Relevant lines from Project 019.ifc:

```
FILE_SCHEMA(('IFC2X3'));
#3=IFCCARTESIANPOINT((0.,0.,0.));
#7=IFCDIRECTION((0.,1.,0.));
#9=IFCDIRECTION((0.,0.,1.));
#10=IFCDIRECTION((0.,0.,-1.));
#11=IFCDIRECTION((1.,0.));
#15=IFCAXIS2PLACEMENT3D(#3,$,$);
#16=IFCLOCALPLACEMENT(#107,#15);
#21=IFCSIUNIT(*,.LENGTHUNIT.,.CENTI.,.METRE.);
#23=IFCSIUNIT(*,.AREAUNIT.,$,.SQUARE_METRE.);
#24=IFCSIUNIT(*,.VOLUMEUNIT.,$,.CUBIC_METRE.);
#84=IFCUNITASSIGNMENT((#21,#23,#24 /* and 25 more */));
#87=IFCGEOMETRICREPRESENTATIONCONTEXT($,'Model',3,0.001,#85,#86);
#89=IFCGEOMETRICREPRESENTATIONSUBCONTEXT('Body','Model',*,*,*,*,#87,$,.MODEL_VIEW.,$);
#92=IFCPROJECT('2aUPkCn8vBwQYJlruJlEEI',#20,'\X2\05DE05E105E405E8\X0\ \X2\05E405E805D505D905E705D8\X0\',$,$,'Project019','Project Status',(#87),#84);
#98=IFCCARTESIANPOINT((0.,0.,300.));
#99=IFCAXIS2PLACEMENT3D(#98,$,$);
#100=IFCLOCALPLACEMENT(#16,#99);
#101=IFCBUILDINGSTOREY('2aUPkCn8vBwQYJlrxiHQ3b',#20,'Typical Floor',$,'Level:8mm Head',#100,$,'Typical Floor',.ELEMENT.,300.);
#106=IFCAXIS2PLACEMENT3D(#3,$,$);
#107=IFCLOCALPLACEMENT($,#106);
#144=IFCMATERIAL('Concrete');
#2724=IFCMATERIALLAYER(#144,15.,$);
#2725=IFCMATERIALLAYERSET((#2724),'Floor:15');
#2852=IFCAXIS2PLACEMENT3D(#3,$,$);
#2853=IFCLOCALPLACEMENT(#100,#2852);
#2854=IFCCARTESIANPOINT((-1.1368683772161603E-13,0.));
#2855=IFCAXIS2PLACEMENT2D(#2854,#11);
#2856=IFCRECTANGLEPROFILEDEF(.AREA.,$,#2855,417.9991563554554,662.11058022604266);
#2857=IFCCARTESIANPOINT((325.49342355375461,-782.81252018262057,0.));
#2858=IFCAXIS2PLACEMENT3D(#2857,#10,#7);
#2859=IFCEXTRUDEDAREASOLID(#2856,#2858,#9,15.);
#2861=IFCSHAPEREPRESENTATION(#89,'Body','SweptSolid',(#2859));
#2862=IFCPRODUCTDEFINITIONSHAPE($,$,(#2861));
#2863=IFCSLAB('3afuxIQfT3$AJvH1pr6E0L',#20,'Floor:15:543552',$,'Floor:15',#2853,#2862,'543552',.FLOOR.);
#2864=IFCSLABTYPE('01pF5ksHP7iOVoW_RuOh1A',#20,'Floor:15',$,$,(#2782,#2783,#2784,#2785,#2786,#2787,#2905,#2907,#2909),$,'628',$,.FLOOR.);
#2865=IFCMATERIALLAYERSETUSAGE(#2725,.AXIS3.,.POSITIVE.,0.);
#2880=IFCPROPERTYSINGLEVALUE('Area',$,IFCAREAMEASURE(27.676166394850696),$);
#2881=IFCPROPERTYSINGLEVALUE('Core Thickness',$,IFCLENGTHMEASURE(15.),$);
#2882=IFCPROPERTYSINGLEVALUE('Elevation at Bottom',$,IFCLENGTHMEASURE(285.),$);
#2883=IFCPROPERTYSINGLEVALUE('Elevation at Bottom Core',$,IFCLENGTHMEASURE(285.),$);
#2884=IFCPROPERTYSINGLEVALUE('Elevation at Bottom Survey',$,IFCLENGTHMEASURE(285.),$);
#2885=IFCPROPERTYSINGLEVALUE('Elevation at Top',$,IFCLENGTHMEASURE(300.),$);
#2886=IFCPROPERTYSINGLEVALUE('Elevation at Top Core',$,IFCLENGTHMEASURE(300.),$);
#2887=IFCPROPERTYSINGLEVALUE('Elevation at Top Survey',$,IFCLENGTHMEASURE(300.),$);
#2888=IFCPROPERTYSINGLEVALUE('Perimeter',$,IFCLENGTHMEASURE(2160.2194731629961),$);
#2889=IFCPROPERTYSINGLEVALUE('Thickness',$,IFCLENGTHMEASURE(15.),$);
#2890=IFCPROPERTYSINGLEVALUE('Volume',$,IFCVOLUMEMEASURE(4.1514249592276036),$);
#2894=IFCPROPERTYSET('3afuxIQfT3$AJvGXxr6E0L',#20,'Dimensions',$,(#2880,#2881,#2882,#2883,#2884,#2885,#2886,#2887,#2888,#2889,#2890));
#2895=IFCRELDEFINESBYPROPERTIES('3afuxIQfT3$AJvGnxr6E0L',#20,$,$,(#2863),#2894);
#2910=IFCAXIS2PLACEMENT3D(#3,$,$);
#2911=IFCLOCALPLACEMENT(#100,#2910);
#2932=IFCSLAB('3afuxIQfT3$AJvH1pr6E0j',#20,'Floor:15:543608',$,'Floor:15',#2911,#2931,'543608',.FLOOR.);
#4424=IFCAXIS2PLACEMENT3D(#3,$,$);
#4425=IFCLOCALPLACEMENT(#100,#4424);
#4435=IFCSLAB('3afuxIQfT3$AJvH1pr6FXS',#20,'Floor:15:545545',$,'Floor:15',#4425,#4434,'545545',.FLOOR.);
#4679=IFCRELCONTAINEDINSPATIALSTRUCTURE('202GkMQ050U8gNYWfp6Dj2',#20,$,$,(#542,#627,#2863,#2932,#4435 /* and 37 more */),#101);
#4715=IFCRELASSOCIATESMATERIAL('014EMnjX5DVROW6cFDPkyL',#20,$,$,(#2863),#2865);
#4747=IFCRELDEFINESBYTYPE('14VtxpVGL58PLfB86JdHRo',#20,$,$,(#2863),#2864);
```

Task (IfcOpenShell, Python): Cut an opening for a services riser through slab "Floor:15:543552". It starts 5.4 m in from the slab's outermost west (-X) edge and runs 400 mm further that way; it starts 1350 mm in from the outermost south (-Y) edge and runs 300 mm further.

```python
import numpy as np
import ifcopenshell
import ifcopenshell.api.feature
import ifcopenshell.api.geometry
import ifcopenshell.api.pset
import ifcopenshell.api.root
import ifcopenshell.geom
import ifcopenshell.util.element
import ifcopenshell.util.placement
import ifcopenshell.util.representation
import ifcopenshell.util.shape
import ifcopenshell.util.unit

model = ifcopenshell.open("Project 019.ifc")
unit_scale = ifcopenshell.util.unit.calculate_unit_scale(model)
area_scale = ifcopenshell.util.unit.calculate_unit_scale(model, "AREAUNIT")
volume_scale = ifcopenshell.util.unit.calculate_unit_scale(model, "VOLUMEUNIT")
settings = ifcopenshell.geom.settings()


def volume(element):
    """Net volume in cubic metres, openings subtracted."""
    shape = ifcopenshell.geom.create_shape(settings, element)
    return ifcopenshell.util.shape.get_volume(shape.geometry)


slab = model.by_guid("3afuxIQfT3$AJvH1pr6E0L")
before = volume(slab)

# Extent in the slab's own axes, in metres. The edges named are its -X and -Y sides.
slab_shape = ifcopenshell.geom.create_shape(settings, slab)
vertices = ifcopenshell.util.shape.get_vertices(slab_shape.geometry)
x_min, y_min, bottom = vertices.min(axis=0)
top = vertices[:, 2].max()

opening = ifcopenshell.api.root.create_entity(model, ifc_class="IfcOpeningElement", name="Services riser opening")
context = ifcopenshell.util.representation.get_context(model, "Model", "Body", "MODEL_VIEW")
width, depth = 0.4, 0.3
outline = [(0.0, 0.0), (width, 0.0), (width, depth), (0.0, depth), (0.0, 0.0)]
# Overshoot both faces by 50 mm so the cut is clean.
shape = ifcopenshell.api.geometry.add_slab_representation(
    model, context=context, depth=top - bottom + 0.1, polyline=outline
)
ifcopenshell.api.geometry.assign_representation(model, product=opening, representation=shape)

matrix = ifcopenshell.util.placement.get_local_placement(slab.ObjectPlacement)
matrix[:, 3] = matrix @ np.append(np.array([x_min + 5.4, y_min + 1.35, bottom - 0.05]) / unit_scale, 1.0)
ifcopenshell.api.geometry.edit_object_placement(model, product=opening, matrix=matrix, is_si=False)
ifcopenshell.api.feature.add_feature(model, feature=opening, element=slab)

after = volume(slab)

# Update the slab's stored quantities.
pset = model.by_id(ifcopenshell.util.element.get_pset(slab, "Dimensions", should_inherit=False)["id"])
ifcopenshell.api.pset.edit_pset(model, pset=pset, properties={
    "Area": model.create_entity("IfcAreaMeasure", after / (top - bottom) / area_scale),
    "Volume": model.create_entity("IfcVolumeMeasure", after / volume_scale),
})

print(f"slab volume {before:.3f} -> {after:.3f} m3")

model.write("Project 019_updated.ifc")
```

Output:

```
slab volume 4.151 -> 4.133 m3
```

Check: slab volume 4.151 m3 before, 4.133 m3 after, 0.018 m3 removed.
